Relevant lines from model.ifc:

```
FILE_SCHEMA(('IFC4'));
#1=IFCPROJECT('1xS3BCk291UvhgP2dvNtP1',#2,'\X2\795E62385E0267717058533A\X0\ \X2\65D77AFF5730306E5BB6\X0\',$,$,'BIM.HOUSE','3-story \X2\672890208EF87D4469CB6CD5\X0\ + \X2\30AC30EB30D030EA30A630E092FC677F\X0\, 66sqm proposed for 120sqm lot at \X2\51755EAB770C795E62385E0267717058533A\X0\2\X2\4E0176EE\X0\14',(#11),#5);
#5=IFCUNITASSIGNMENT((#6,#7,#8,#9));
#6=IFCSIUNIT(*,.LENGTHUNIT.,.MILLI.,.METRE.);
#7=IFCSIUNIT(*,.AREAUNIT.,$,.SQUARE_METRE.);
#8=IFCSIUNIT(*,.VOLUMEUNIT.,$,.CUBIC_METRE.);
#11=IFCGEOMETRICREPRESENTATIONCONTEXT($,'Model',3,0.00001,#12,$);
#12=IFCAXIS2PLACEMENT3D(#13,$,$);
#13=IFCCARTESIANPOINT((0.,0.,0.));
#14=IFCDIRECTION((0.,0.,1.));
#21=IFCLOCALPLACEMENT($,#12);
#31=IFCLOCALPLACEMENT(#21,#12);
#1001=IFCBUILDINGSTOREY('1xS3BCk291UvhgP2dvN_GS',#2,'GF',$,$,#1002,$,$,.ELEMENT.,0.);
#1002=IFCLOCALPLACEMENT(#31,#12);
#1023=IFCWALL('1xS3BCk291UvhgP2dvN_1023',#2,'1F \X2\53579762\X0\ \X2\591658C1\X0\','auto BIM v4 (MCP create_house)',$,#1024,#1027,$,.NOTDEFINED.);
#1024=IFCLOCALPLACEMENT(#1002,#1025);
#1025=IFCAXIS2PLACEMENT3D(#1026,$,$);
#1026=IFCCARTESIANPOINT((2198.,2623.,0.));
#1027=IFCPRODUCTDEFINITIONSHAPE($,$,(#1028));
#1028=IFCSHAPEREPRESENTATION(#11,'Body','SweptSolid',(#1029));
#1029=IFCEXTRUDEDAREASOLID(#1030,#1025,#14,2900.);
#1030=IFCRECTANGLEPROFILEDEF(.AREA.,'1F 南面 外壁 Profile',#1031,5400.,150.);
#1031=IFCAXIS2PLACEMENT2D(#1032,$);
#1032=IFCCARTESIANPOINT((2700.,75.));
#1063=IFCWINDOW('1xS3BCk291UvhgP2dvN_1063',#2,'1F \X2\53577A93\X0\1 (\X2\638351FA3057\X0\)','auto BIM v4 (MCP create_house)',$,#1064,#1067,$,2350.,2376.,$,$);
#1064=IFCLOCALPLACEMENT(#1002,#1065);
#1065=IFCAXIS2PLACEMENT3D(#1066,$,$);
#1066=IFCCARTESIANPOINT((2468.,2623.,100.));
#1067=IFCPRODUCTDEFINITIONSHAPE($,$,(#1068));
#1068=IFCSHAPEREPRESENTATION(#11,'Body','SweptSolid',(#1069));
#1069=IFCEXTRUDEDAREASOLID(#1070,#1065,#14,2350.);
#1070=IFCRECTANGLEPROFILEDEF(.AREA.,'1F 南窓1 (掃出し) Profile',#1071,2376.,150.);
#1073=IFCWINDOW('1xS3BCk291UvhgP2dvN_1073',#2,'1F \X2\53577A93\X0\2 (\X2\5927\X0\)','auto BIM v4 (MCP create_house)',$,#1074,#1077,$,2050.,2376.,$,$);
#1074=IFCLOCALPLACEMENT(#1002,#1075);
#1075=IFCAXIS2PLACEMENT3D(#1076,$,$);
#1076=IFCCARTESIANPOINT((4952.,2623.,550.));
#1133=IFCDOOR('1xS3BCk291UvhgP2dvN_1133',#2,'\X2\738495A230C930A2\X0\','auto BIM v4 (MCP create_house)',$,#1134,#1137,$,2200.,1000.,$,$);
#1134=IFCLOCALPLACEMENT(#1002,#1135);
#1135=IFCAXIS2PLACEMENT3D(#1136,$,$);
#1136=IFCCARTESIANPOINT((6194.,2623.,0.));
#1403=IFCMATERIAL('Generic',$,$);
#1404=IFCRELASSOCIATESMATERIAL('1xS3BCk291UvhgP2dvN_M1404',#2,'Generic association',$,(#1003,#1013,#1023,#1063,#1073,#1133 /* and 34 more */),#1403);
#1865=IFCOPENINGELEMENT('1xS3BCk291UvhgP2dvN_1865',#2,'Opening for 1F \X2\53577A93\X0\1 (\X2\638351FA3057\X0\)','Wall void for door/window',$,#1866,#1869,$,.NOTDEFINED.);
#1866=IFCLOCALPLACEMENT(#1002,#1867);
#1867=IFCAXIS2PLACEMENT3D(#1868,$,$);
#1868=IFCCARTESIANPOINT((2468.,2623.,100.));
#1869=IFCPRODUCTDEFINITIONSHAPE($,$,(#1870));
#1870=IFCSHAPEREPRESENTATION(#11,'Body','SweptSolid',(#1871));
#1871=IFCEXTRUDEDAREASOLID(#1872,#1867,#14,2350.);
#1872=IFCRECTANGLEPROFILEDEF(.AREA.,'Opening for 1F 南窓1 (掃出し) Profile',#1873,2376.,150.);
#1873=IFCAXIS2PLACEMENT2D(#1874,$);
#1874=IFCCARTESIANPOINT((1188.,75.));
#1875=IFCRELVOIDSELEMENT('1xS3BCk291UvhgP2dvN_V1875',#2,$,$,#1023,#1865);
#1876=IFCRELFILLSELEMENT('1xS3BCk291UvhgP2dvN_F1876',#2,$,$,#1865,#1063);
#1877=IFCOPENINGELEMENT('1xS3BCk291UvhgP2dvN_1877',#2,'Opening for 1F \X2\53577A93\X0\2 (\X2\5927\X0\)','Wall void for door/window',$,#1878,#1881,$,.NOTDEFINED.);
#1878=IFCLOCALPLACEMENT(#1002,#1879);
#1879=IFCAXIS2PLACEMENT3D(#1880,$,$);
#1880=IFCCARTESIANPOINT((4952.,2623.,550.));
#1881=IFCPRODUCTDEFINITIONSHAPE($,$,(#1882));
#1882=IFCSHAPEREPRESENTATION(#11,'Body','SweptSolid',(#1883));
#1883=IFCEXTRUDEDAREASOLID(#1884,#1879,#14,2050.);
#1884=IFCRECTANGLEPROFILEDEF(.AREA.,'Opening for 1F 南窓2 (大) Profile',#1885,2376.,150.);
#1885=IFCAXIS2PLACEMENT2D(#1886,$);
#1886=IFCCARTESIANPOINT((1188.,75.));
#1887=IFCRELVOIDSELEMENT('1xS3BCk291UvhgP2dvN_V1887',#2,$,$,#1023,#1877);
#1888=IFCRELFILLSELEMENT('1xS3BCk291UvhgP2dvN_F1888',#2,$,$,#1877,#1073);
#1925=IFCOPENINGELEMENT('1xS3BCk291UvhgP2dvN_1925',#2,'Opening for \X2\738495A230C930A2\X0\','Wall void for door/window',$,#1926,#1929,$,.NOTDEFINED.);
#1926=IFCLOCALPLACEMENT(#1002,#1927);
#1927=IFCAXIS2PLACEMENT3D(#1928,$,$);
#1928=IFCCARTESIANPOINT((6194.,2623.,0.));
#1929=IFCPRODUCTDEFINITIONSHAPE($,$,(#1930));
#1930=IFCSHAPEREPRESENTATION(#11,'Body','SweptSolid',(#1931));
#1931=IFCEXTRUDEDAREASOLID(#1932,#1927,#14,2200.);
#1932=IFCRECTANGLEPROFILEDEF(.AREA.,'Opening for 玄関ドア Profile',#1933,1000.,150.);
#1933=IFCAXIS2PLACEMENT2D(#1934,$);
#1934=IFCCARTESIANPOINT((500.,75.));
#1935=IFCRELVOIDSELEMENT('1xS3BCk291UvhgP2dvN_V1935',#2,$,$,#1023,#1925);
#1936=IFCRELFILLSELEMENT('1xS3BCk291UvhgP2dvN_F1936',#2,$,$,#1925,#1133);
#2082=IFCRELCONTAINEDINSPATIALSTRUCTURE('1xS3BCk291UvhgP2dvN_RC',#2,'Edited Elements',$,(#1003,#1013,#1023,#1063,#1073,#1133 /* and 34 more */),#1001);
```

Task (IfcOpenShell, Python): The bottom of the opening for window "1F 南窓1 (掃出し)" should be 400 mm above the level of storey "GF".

```python
import numpy as np
import ifcopenshell
import ifcopenshell.api.geometry
import ifcopenshell.geom
import ifcopenshell.util.element
import ifcopenshell.util.placement
import ifcopenshell.util.shape
import ifcopenshell.util.unit

model = ifcopenshell.open("model.ifc")
unit_scale = ifcopenshell.util.unit.calculate_unit_scale(model)

window = model.by_id(1063)
opening = window.FillsVoids[0].RelatingOpeningElement
storey = ifcopenshell.util.element.get_container(window, ifc_class="IfcBuildingStorey")
level = ifcopenshell.util.placement.get_local_placement(storey.ObjectPlacement)[2, 3]

# The opening's origin need not be at the sill, so measure its lowest point.
shape = ifcopenshell.geom.create_shape(ifcopenshell.geom.settings(), opening)
bottom = ifcopenshell.util.shape.get_shape_bottom_elevation(shape, shape.geometry) / unit_scale
dz = level + 0.4 / unit_scale - bottom

shift = np.array([0.0, 0.0, dz])
# The window is not placed relative to its opening, so move both.
for product in (opening, window):
    matrix = ifcopenshell.util.placement.get_local_placement(product.ObjectPlacement)
    matrix[:3, 3] += shift
    ifcopenshell.api.geometry.edit_object_placement(model, product=product, matrix=matrix, is_si=False)

print(f"moved by {dz * unit_scale:+.3f} m")

model.write("model_v2.ifc")
```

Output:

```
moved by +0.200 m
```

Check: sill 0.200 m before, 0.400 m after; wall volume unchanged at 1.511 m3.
